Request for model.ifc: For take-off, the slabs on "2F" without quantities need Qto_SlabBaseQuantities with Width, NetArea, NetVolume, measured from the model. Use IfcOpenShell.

First a look at what the model holds.

```python
import ifcopenshell
import ifcopenshell.util.element
import ifcopenshell.util.unit

model = ifcopenshell.open("model.ifc")
print(model.schema)
for unit_type in ("LENGTHUNIT", "AREAUNIT", "VOLUMEUNIT"):
    print(unit_type, ifcopenshell.util.unit.calculate_unit_scale(model, unit_type))
storey = next(s for s in model.by_type("IfcBuildingStorey") if s.Name == "2F")
slabs = [e for e in ifcopenshell.util.element.get_decomposition(storey) if e.is_a("IfcSlab")]
for e in sorted(slabs, key=lambda e: e.id()):
    print(e.id(), e.is_a(), e.Name, list(ifcopenshell.util.element.get_psets(e, qtos_only=True)), sep=" | ")
```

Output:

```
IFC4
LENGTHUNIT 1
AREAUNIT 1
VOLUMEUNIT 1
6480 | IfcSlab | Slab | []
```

```python
import ifcopenshell
import ifcopenshell.api.pset
import ifcopenshell.geom
import ifcopenshell.util.element
import ifcopenshell.util.shape
import ifcopenshell.util.unit

model = ifcopenshell.open("model.ifc")
unit_scale = ifcopenshell.util.unit.calculate_unit_scale(model)
area_scale = ifcopenshell.util.unit.calculate_unit_scale(model, "AREAUNIT")
volume_scale = ifcopenshell.util.unit.calculate_unit_scale(model, "VOLUMEUNIT")
settings = ifcopenshell.geom.settings()

storey = next(s for s in model.by_type("IfcBuildingStorey") if s.Name == "2F")
slabs = [e for e in ifcopenshell.util.element.get_decomposition(storey) if e.is_a("IfcSlab")]

for e in sorted(slabs, key=lambda e: e.id()):
    if ifcopenshell.util.element.get_psets(e, qtos_only=True, should_inherit=False):
        continue
    # Geometry comes back in metres, in the element's own axes.
    shape = ifcopenshell.geom.create_shape(settings, e)
    values = {
        "Width": ifcopenshell.util.shape.get_z(shape.geometry) / unit_scale,
        "NetArea": ifcopenshell.util.shape.get_footprint_area(shape.geometry) / area_scale,
        "NetVolume": ifcopenshell.util.shape.get_volume(shape.geometry) / volume_scale,
    }
    qto = ifcopenshell.api.pset.add_qto(model, product=e, name="Qto_SlabBaseQuantities")
    ifcopenshell.api.pset.edit_qto(model, qto=qto, properties=values)
    print(e.id(), {k: round(v, 3) for k, v in values.items()})

model.write("model_edited.ifc")
```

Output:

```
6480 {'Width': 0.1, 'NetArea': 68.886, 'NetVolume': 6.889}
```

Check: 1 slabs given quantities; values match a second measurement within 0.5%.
